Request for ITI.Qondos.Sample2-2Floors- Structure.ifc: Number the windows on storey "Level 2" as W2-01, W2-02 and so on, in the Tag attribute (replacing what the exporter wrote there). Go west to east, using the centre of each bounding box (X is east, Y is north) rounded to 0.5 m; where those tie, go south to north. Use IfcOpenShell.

First a look at what the model holds.

```python
import ifcopenshell
import ifcopenshell.util.element
import ifcopenshell.util.placement

model = ifcopenshell.open("ITI.Qondos.Sample2-2Floors- Structure.ifc")
print(model.schema)
storey = next(s for s in model.by_type("IfcBuildingStorey") if s.Name == "Level 2")
windows = [e for e in ifcopenshell.util.element.get_decomposition(storey) if e.is_a("IfcWindow")]
for e in sorted(windows, key=lambda e: e.id()):
    origin = ifcopenshell.util.placement.get_local_placement(e.ObjectPlacement)[:3, 3]
    print(e.id(), e.Tag, e.Name, origin.round(2) + 0.0, sep=" | ")
```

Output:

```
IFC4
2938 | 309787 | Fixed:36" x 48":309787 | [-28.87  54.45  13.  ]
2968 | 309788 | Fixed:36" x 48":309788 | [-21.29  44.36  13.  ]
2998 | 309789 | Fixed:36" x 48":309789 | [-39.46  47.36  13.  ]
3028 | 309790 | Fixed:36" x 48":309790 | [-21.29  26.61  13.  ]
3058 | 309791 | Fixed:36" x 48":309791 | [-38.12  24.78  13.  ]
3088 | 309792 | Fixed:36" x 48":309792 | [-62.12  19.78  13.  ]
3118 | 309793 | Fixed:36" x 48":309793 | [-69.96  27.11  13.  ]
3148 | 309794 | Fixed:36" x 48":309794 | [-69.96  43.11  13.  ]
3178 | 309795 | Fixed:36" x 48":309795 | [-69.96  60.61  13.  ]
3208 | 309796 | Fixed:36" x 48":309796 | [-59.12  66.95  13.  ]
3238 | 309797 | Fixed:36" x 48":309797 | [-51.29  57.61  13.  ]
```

```python
import ifcopenshell
import ifcopenshell.geom
import ifcopenshell.util.element
import ifcopenshell.util.shape

model = ifcopenshell.open("ITI.Qondos.Sample2-2Floors- Structure.ifc")
settings = ifcopenshell.geom.settings()
settings.set("use-world-coords", True)


def centre(element):
    shape = ifcopenshell.geom.create_shape(settings, element)
    return ifcopenshell.util.shape.get_bbox_centroid(shape.geometry)


storey = next(s for s in model.by_type("IfcBuildingStorey") if s.Name == "Level 2")
windows = [e for e in ifcopenshell.util.element.get_decomposition(storey) if e.is_a("IfcWindow")]

# Insertion points can sit at a corner or the storey origin, so sort by the geometry (in metres).
centres = {e: centre(e) for e in windows}
windows.sort(key=lambda e: (round(centres[e][0] / 0.5), centres[e][1]))

for i, e in enumerate(windows, start=1):
    number = f"W2-{i:02d}"
    e.Tag = number
    print(e.id(), number)

model.write("ITI.Qondos.Sample2-2Floors- Structure_v2.ifc")
```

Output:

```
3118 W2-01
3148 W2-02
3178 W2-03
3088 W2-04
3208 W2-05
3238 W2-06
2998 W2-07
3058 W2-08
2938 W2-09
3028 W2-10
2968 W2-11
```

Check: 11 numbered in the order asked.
